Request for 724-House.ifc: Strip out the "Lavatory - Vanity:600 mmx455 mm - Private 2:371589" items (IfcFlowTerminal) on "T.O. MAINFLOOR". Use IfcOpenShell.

First a look at what the model holds.

```python
import ifcopenshell
import ifcopenshell.util.element

model = ifcopenshell.open("724-House.ifc")
print(model.schema)
storey = next(s for s in model.by_type("IfcBuildingStorey") if s.Name == "T.O. MAINFLOOR")
terminals = [e for e in ifcopenshell.util.element.get_decomposition(storey) if e.is_a("IfcFlowTerminal")]
seen = {}
for e in terminals:
    element_type = ifcopenshell.util.element.get_type(e)
    name = element_type.Name if element_type not in (None, e) else None
    seen[name] = seen.get(name, 0) + 1
for name, count in sorted(seen.items(), key=str):
    print(count, "x", name)
```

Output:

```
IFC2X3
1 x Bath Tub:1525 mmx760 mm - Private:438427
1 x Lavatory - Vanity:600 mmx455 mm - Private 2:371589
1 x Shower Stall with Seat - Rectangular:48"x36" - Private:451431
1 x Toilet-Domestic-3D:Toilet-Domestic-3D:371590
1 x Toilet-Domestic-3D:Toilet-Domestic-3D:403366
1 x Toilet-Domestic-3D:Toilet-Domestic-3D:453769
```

```python
import ifcopenshell
import ifcopenshell.api.root
import ifcopenshell.util.element

model = ifcopenshell.open("724-House.ifc")

storey = next(s for s in model.by_type("IfcBuildingStorey") if s.Name == "T.O. MAINFLOOR")
terminals = [e for e in ifcopenshell.util.element.get_decomposition(storey) if e.is_a("IfcFlowTerminal")]
targets = [e for e in terminals if (t := ifcopenshell.util.element.get_type(e)) not in (None, e) and t.Name == "Lavatory - Vanity:600 mmx455 mm - Private 2:371589"]

for e in targets:
    ifcopenshell.api.root.remove_product(model, product=e)
print(len(targets), "removed")

model.write("724-House_rev.ifc")
```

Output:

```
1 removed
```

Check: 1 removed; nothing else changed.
